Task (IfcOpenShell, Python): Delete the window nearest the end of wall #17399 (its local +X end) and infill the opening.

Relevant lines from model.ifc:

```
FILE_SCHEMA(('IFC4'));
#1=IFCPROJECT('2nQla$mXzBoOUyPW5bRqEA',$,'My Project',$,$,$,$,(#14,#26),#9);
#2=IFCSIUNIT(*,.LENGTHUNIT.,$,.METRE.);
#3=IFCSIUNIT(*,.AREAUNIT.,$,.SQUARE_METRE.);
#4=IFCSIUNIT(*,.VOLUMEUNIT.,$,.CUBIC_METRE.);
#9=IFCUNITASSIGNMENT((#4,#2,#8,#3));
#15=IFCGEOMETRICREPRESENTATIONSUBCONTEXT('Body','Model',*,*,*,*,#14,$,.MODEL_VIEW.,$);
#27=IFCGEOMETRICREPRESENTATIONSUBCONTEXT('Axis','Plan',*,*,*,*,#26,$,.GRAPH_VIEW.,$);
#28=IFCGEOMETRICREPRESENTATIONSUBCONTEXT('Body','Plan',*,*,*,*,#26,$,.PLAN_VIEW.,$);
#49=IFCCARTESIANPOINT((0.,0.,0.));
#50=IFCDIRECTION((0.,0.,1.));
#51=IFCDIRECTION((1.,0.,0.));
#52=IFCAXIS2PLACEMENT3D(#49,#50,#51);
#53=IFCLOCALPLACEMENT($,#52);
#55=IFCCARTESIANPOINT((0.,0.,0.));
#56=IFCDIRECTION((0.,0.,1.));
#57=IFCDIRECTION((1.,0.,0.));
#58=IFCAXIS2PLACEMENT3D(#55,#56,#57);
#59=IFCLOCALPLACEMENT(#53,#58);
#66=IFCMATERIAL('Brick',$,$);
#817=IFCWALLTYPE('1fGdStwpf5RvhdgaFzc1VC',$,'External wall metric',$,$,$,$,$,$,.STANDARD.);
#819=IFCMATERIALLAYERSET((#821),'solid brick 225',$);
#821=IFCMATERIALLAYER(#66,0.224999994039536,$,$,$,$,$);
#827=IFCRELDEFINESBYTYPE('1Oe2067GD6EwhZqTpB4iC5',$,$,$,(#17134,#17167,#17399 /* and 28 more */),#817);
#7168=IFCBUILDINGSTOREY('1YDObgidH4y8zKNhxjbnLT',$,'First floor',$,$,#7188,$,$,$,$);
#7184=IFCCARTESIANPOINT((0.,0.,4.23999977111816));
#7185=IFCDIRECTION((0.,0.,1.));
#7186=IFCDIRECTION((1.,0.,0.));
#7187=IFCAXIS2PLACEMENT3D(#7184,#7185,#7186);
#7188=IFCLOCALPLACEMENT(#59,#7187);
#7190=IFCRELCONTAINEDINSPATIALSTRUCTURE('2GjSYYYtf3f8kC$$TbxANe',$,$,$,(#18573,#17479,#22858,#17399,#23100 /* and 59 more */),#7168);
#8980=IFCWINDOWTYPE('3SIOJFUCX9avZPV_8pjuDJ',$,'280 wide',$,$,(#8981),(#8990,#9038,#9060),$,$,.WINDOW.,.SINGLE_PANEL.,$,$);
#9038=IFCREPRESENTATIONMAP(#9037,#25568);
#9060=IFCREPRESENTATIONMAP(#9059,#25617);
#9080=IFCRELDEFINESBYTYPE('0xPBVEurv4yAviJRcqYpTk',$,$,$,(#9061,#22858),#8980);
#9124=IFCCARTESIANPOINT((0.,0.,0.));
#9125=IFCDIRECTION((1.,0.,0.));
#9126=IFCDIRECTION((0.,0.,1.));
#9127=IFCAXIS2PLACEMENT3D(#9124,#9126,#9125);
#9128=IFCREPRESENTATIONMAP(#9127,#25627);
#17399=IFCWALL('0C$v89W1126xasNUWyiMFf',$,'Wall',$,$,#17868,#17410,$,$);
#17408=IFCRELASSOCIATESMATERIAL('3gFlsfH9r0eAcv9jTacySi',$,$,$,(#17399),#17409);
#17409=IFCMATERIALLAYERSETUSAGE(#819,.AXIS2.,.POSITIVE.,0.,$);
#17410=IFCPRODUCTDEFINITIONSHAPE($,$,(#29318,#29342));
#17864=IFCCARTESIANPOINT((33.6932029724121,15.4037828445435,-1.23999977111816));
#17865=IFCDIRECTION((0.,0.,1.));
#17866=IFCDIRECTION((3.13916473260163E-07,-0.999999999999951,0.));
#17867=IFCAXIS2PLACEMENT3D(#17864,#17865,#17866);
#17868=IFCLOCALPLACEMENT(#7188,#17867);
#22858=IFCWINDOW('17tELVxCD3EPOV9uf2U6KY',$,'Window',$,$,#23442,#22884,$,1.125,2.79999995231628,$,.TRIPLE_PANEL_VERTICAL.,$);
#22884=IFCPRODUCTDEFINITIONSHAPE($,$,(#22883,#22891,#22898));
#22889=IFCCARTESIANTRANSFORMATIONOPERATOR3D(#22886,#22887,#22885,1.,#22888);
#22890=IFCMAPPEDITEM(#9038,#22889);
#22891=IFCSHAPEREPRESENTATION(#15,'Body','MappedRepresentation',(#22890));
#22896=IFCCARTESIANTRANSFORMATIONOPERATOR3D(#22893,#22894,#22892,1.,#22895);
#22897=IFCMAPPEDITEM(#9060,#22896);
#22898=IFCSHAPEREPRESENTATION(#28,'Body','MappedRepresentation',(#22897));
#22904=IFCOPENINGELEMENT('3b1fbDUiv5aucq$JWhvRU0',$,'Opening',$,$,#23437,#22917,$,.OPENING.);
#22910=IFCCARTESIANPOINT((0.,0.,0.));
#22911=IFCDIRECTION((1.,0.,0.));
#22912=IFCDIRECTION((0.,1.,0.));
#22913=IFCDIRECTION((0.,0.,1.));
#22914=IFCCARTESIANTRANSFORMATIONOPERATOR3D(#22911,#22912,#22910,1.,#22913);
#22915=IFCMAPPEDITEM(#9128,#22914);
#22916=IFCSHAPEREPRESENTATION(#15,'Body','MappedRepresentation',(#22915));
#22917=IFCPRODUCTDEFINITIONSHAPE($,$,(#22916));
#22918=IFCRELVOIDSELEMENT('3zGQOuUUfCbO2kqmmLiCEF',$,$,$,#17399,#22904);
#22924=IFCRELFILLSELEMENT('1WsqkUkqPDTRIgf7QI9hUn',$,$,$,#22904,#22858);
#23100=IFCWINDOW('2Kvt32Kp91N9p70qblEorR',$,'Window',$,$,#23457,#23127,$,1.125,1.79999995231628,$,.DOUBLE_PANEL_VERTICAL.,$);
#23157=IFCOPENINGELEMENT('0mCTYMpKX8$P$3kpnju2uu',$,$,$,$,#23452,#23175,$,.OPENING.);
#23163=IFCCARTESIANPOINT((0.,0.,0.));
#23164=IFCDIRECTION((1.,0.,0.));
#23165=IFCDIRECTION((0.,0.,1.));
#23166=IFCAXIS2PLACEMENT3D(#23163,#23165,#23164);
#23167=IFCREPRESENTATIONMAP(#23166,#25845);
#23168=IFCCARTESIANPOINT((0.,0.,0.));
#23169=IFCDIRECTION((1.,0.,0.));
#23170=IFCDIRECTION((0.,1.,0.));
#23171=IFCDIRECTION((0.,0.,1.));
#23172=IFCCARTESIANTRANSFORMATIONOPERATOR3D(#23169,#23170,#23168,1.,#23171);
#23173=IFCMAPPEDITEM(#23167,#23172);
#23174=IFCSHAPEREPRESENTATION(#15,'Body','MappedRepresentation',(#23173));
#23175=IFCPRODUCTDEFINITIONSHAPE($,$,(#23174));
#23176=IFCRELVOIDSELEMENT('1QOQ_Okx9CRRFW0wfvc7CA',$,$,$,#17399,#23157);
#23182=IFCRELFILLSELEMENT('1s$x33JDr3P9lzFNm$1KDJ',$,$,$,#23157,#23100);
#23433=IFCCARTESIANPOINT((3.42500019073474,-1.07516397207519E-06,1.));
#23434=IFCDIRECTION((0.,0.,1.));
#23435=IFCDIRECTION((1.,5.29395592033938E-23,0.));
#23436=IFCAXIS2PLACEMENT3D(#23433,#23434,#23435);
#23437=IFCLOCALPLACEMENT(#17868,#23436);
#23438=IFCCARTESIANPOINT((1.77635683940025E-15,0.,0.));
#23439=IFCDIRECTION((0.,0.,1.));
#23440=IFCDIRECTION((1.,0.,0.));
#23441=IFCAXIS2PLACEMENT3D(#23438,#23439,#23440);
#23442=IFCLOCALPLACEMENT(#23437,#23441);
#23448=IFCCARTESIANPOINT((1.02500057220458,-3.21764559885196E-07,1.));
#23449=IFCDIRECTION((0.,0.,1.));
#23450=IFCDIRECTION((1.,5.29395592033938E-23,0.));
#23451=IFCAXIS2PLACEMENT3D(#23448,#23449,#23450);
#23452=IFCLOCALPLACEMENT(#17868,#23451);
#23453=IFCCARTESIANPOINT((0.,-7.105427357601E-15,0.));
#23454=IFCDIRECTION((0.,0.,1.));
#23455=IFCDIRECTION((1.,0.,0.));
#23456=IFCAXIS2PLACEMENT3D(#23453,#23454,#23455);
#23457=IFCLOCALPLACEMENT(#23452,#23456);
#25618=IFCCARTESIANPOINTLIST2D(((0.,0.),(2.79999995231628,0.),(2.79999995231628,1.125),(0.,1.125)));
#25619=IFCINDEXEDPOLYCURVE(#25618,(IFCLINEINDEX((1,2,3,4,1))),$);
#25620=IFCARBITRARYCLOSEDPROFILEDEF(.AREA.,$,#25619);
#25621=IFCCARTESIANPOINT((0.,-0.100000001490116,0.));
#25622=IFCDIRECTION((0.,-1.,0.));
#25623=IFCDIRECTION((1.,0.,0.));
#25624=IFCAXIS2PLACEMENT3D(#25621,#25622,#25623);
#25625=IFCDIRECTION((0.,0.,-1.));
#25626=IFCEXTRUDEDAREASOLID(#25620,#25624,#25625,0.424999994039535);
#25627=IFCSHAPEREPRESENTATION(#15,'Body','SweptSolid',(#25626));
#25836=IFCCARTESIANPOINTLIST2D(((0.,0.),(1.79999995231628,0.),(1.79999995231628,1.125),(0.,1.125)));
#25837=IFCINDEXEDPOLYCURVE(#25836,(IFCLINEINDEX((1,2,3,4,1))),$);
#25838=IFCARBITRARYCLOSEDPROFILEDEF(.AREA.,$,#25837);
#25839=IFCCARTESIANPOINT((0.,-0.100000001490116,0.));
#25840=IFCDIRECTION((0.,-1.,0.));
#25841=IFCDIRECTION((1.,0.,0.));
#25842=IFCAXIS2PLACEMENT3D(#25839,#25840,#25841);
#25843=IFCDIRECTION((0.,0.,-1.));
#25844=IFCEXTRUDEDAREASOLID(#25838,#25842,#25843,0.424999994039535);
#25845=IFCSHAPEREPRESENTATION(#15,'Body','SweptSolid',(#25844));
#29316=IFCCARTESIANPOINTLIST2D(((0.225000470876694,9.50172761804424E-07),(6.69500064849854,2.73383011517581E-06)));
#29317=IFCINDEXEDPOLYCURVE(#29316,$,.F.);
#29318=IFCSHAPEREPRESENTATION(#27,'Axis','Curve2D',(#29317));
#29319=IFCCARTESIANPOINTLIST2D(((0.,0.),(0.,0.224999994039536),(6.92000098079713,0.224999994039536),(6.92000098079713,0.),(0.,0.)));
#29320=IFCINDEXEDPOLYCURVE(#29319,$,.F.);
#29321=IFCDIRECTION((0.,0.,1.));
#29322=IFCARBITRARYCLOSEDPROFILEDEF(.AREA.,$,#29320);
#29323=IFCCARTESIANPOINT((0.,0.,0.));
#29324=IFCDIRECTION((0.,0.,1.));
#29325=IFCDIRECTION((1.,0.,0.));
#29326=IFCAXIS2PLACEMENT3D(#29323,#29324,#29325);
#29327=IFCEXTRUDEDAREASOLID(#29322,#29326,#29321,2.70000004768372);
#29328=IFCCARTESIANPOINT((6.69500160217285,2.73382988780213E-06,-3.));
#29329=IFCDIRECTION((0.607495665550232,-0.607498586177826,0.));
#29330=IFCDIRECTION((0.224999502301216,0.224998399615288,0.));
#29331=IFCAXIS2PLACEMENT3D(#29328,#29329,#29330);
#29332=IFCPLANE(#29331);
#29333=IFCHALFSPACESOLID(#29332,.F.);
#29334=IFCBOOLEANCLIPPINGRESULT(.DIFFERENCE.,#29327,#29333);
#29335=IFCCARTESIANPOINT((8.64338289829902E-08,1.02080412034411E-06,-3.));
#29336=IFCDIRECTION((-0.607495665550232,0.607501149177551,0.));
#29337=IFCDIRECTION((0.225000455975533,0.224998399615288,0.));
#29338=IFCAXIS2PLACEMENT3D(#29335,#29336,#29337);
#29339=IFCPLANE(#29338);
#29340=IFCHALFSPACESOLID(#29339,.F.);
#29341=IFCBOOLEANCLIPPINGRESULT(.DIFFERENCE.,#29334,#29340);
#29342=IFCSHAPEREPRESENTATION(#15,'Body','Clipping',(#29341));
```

```python
import ifcopenshell
import ifcopenshell.api.feature
import ifcopenshell.api.root
import ifcopenshell.geom
import ifcopenshell.util.shape

model = ifcopenshell.open("model.ifc")
settings = ifcopenshell.geom.settings()


def volume(element):
    """Net volume in cubic metres, openings subtracted."""
    shape = ifcopenshell.geom.create_shape(settings, element)
    return ifcopenshell.util.shape.get_volume(shape.geometry)


window = model.by_guid("17tELVxCD3EPOV9uf2U6KY")
opening = window.FillsVoids[0].RelatingOpeningElement
wall = opening.VoidsElements[0].RelatingBuildingElement
before = volume(wall)

ifcopenshell.api.root.remove_product(model, product=window)
ifcopenshell.api.feature.remove_feature(model, feature=opening)

after = volume(wall)

print(f"wall volume {before:.3f} -> {after:.3f} m3")

model.write("model_updated.ifc")
```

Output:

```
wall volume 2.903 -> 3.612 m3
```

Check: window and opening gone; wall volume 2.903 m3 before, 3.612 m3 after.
